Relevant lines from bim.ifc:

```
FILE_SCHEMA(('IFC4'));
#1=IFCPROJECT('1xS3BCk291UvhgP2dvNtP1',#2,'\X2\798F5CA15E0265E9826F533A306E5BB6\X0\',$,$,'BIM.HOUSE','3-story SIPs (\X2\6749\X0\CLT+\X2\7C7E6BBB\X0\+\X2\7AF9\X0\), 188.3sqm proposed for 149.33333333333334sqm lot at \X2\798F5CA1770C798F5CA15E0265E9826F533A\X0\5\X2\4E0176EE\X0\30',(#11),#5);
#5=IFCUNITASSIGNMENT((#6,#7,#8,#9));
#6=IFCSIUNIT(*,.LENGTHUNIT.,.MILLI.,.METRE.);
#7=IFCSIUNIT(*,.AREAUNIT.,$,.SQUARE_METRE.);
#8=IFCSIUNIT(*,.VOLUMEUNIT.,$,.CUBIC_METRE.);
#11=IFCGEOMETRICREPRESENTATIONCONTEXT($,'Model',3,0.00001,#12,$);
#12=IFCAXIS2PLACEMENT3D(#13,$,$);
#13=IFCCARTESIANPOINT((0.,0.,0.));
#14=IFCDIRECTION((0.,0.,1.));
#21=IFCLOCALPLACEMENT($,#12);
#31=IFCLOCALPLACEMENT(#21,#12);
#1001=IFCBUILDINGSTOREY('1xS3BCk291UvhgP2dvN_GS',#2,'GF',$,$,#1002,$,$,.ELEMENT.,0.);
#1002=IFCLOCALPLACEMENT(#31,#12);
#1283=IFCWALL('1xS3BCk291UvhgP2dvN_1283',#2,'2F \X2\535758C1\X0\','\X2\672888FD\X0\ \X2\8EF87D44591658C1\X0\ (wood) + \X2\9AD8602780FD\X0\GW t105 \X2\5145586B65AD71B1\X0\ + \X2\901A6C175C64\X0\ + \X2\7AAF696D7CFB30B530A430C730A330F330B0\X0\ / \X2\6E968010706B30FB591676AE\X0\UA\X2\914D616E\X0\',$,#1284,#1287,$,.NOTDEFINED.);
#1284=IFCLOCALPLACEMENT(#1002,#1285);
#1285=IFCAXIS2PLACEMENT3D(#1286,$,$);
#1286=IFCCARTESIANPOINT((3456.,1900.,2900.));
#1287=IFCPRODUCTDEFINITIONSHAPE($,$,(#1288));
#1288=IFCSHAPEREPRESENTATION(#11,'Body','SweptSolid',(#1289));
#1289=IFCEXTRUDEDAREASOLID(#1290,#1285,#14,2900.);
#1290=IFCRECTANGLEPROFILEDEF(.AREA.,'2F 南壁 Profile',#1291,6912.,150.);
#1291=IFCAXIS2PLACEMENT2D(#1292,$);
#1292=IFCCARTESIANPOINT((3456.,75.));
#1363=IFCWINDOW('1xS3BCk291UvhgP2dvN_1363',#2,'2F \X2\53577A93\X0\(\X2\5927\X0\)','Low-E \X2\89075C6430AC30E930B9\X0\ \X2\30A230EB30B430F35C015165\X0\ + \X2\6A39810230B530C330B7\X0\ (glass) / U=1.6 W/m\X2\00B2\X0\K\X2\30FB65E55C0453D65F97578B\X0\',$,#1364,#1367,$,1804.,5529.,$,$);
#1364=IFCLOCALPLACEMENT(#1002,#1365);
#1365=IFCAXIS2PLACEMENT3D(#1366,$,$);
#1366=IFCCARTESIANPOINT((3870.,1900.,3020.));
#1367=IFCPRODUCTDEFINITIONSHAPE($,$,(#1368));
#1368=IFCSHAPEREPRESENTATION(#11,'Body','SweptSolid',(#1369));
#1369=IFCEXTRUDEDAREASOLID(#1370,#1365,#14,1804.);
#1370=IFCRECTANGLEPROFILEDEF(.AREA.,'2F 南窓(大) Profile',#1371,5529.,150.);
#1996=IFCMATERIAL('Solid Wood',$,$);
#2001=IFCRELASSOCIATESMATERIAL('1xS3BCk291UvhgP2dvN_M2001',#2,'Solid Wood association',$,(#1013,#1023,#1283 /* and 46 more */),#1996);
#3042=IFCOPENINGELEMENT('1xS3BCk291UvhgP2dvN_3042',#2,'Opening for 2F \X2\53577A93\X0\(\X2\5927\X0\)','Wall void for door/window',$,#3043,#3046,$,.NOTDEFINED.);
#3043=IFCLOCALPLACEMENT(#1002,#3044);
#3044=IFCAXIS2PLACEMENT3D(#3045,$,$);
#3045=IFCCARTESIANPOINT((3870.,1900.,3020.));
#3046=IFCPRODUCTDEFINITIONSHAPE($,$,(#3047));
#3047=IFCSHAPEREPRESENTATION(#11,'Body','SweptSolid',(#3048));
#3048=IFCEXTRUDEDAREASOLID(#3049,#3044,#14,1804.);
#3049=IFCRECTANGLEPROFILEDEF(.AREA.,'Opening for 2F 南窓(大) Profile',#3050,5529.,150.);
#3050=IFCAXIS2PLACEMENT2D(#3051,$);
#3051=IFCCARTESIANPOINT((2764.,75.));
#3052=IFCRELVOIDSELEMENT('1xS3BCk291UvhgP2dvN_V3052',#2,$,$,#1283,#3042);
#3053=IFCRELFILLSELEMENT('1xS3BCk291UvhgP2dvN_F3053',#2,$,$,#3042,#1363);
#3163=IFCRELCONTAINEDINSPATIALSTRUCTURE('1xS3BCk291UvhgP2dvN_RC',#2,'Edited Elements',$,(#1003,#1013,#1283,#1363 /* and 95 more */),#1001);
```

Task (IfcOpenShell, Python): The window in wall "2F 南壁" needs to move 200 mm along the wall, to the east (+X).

```python
import ifcopenshell
import ifcopenshell.api.geometry
import ifcopenshell.util.placement
import ifcopenshell.util.unit

model = ifcopenshell.open("bim.ifc")
unit_scale = ifcopenshell.util.unit.calculate_unit_scale(model)

window = model.by_id(1363)
opening = window.FillsVoids[0].RelatingOpeningElement
wall = opening.VoidsElements[0].RelatingBuildingElement

wall_matrix = ifcopenshell.util.placement.get_local_placement(wall.ObjectPlacement)
shift = wall_matrix[:3, 0] * 0.2 / unit_scale
before = ifcopenshell.util.placement.get_local_placement(window.ObjectPlacement)[:3, 3].copy()

# The window is not placed relative to its opening, so move both.
for product in (opening, window):
    matrix = ifcopenshell.util.placement.get_local_placement(product.ObjectPlacement)
    matrix[:3, 3] += shift
    ifcopenshell.api.geometry.edit_object_placement(model, product=product, matrix=matrix, is_si=False)

after = ifcopenshell.util.placement.get_local_placement(window.ObjectPlacement)[:3, 3]
print("window moved by", (after - before).round(3) + 0.0)

model.write("bim-out.ifc")
```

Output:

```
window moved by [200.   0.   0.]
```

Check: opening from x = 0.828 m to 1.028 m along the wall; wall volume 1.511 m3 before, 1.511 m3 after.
